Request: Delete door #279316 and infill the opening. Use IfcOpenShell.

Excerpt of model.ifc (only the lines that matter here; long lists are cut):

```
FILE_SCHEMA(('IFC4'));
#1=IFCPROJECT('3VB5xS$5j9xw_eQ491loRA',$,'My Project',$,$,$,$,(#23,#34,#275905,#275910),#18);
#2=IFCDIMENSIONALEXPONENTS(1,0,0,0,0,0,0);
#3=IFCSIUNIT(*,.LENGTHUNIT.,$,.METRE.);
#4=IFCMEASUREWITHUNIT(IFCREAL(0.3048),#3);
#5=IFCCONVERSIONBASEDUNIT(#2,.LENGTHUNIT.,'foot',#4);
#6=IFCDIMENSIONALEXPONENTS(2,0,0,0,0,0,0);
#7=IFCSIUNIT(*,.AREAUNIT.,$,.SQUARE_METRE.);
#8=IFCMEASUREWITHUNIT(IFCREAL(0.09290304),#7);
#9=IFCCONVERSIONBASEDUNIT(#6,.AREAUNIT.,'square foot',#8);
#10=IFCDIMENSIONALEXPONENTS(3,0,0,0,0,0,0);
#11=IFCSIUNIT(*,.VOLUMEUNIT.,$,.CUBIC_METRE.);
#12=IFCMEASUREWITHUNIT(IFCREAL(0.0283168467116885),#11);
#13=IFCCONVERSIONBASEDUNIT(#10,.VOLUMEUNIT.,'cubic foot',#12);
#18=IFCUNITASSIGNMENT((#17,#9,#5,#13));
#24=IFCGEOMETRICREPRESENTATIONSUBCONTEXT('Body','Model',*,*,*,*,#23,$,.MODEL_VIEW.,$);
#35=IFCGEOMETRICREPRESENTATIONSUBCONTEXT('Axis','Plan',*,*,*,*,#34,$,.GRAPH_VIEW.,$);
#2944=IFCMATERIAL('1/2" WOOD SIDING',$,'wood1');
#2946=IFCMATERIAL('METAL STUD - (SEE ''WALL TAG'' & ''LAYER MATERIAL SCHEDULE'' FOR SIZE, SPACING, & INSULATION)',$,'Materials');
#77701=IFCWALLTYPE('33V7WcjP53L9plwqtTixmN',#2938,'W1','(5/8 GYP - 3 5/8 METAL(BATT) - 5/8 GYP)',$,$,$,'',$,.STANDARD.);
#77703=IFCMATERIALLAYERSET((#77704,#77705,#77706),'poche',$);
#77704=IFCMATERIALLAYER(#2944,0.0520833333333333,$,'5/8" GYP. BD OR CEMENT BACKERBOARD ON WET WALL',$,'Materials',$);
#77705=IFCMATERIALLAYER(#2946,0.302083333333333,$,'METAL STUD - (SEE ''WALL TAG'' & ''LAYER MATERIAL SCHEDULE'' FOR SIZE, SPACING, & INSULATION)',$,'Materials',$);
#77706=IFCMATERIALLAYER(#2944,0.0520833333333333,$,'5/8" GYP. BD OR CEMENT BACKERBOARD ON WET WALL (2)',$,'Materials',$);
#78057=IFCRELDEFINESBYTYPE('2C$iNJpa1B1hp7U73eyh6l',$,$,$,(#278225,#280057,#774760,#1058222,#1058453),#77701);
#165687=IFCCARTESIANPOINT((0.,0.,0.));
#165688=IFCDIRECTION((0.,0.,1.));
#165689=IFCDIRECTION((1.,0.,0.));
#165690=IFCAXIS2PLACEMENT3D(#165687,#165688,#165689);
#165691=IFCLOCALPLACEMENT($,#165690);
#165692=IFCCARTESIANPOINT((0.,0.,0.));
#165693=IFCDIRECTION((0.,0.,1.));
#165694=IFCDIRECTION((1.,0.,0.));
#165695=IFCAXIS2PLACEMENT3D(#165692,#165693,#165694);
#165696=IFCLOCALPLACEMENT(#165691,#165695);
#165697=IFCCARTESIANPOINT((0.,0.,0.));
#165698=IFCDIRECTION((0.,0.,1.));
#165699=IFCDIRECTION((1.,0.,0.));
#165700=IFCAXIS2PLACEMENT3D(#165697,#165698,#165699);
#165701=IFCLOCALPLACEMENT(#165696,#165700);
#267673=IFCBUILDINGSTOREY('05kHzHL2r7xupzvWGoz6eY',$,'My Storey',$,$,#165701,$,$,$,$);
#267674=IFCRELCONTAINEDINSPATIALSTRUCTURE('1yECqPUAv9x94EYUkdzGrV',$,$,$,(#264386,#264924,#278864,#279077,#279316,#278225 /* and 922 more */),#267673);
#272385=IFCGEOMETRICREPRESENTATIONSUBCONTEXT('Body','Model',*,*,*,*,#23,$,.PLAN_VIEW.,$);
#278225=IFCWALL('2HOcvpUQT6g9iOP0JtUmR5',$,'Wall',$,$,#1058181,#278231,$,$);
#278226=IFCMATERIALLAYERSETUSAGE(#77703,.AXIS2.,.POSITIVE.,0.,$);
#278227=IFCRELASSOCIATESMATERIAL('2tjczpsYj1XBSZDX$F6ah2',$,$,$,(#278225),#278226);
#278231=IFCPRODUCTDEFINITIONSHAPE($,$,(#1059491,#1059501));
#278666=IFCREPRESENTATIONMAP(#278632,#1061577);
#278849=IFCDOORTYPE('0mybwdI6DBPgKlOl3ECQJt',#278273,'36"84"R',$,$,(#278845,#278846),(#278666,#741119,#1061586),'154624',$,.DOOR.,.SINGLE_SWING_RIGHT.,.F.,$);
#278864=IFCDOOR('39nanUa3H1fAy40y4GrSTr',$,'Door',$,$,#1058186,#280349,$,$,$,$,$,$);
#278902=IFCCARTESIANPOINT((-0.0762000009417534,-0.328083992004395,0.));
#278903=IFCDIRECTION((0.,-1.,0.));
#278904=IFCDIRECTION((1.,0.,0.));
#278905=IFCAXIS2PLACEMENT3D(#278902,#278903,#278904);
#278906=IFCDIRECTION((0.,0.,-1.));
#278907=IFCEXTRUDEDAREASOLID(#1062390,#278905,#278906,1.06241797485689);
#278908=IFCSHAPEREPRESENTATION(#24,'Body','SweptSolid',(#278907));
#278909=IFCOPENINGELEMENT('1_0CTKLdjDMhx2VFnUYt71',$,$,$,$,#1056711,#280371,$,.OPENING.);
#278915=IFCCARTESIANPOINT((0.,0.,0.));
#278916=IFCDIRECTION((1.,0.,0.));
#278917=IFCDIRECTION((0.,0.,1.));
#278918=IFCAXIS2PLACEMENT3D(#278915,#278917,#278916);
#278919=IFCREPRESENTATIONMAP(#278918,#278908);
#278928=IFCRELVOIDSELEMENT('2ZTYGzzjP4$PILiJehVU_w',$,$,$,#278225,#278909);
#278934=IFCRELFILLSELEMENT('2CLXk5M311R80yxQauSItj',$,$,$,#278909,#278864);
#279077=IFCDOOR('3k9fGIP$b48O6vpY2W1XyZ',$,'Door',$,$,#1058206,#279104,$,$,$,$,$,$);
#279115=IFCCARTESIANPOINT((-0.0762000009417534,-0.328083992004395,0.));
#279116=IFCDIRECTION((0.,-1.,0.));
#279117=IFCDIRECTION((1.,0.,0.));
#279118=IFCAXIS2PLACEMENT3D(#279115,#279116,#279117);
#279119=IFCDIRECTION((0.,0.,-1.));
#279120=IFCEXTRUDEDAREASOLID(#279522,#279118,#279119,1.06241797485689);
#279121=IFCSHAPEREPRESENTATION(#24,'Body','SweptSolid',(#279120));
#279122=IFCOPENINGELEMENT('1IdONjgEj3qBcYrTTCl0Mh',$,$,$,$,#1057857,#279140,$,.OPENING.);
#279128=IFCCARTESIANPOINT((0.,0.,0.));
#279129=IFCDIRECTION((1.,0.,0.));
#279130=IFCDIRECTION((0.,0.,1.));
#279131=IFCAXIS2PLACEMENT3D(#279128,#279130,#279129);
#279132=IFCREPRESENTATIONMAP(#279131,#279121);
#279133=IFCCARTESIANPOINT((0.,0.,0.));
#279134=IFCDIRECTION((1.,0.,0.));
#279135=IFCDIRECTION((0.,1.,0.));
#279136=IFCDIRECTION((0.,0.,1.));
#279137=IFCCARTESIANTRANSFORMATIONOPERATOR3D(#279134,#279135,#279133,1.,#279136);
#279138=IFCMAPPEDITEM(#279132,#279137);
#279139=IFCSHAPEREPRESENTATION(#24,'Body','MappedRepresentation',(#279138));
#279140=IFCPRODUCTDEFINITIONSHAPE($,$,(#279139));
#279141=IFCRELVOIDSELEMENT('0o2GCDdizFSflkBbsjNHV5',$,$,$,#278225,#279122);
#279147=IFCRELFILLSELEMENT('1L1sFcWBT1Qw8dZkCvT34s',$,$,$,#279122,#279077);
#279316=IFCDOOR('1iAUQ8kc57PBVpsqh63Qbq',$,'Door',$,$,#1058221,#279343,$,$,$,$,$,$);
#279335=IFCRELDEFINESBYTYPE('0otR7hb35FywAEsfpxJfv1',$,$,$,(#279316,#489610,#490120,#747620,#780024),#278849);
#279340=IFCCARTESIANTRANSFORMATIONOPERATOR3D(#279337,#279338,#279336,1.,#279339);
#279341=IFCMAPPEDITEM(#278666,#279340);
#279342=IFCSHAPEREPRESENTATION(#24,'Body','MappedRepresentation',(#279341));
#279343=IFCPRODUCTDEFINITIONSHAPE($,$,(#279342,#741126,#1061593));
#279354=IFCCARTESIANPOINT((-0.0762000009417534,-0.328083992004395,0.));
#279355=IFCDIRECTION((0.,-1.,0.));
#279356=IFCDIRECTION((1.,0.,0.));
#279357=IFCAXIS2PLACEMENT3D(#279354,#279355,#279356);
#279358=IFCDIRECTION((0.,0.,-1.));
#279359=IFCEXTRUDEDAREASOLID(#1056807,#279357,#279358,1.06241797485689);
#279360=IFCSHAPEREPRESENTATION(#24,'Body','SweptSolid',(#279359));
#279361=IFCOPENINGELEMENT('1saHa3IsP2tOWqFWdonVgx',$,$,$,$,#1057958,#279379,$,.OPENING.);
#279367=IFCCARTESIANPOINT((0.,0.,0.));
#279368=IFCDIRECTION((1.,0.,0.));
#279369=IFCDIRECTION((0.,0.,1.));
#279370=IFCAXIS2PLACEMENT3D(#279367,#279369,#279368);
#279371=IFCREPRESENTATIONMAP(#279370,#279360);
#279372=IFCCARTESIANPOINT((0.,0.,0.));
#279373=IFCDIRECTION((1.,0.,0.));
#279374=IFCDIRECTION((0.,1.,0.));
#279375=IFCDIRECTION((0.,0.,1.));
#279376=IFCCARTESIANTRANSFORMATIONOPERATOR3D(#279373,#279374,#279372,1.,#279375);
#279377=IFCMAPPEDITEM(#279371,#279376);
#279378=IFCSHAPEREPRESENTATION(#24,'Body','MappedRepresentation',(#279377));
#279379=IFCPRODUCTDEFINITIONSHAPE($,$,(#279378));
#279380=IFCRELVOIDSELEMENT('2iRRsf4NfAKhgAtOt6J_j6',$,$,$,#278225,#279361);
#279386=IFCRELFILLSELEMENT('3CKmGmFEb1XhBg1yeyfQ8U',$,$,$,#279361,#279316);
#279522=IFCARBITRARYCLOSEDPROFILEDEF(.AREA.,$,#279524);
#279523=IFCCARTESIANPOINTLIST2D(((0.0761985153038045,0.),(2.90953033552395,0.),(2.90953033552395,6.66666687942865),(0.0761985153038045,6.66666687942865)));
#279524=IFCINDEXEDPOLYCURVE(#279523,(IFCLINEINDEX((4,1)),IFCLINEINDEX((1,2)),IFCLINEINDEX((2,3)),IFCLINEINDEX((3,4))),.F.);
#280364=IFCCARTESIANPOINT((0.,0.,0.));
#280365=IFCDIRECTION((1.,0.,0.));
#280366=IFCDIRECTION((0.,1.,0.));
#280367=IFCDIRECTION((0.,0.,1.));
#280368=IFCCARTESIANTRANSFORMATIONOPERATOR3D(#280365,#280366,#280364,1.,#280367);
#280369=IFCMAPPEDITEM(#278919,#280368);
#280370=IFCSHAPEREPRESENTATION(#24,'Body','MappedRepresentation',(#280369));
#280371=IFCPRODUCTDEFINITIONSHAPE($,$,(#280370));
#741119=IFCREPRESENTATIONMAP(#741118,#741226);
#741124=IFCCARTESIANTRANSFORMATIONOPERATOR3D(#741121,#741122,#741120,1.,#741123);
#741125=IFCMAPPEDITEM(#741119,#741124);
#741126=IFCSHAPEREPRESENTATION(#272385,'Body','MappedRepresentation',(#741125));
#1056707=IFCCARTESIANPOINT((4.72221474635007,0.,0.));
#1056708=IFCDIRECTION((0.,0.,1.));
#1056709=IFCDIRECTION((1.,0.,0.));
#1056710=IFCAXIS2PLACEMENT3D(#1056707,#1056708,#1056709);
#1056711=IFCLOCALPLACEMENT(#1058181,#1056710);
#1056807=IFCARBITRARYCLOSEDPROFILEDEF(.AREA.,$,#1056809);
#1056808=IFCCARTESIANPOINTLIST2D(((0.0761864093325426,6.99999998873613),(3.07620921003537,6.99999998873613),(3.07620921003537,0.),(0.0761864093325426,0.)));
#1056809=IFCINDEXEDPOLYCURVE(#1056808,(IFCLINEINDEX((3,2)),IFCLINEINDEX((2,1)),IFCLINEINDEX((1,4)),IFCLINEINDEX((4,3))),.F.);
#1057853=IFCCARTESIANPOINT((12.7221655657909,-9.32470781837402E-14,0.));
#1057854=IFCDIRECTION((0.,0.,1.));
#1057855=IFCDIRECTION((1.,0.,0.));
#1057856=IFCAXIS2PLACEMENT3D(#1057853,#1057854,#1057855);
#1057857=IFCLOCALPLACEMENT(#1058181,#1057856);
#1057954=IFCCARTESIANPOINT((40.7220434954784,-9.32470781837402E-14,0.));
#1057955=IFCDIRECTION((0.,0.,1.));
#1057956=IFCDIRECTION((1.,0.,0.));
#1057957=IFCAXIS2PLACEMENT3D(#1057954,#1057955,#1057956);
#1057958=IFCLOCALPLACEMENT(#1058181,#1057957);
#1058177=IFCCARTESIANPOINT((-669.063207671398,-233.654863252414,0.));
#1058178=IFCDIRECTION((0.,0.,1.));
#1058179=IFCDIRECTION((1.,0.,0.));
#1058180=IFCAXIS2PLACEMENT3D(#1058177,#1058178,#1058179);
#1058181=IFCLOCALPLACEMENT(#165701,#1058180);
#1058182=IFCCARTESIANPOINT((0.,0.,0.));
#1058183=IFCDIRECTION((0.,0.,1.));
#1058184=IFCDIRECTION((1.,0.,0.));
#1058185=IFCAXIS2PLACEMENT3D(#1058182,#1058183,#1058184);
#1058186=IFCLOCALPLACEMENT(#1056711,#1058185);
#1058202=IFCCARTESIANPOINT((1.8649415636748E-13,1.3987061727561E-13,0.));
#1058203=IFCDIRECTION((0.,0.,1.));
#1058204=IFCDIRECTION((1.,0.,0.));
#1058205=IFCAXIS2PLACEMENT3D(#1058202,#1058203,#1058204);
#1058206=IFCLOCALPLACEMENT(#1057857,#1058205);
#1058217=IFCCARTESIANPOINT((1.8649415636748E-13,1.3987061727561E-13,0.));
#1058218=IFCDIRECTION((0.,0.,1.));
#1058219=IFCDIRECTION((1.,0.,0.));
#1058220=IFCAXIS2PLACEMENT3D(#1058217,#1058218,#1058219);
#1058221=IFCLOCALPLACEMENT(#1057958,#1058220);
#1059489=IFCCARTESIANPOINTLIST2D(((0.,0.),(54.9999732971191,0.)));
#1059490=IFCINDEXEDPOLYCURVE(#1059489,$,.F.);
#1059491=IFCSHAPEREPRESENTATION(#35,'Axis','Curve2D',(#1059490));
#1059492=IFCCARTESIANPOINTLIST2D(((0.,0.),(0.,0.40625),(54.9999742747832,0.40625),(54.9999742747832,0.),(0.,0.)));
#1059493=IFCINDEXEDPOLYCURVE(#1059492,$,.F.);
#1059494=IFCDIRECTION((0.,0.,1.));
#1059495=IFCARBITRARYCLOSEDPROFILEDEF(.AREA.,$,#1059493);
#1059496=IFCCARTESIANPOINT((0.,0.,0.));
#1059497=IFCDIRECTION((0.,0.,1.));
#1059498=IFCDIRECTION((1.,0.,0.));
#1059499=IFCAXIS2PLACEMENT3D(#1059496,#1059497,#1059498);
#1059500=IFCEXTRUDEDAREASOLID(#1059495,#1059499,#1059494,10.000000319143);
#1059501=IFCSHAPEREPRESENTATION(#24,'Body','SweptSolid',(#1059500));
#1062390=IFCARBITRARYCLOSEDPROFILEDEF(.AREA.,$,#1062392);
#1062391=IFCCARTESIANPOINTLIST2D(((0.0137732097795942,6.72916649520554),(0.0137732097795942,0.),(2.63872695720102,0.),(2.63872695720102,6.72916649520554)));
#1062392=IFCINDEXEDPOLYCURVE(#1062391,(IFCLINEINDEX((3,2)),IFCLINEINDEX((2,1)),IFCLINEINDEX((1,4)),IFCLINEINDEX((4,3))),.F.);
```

```python
import ifcopenshell
import ifcopenshell.api.feature
import ifcopenshell.api.root
import ifcopenshell.geom
import ifcopenshell.util.shape

model = ifcopenshell.open("model.ifc")
settings = ifcopenshell.geom.settings()


def volume(element):
    """Net volume in cubic metres, openings subtracted."""
    shape = ifcopenshell.geom.create_shape(settings, element)
    return ifcopenshell.util.shape.get_volume(shape.geometry)


door = model.by_guid("1iAUQ8kc57PBVpsqh63Qbq")
opening = door.FillsVoids[0].RelatingOpeningElement
wall = opening.VoidsElements[0].RelatingBuildingElement
before = volume(wall)

ifcopenshell.api.root.remove_product(model, product=door)
ifcopenshell.api.feature.remove_feature(model, feature=opening)

after = volume(wall)

print(f"wall volume {before:.3f} -> {after:.3f} m3")

model.write("model-out.ifc")
```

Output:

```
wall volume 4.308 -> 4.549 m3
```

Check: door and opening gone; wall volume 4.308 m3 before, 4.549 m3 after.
